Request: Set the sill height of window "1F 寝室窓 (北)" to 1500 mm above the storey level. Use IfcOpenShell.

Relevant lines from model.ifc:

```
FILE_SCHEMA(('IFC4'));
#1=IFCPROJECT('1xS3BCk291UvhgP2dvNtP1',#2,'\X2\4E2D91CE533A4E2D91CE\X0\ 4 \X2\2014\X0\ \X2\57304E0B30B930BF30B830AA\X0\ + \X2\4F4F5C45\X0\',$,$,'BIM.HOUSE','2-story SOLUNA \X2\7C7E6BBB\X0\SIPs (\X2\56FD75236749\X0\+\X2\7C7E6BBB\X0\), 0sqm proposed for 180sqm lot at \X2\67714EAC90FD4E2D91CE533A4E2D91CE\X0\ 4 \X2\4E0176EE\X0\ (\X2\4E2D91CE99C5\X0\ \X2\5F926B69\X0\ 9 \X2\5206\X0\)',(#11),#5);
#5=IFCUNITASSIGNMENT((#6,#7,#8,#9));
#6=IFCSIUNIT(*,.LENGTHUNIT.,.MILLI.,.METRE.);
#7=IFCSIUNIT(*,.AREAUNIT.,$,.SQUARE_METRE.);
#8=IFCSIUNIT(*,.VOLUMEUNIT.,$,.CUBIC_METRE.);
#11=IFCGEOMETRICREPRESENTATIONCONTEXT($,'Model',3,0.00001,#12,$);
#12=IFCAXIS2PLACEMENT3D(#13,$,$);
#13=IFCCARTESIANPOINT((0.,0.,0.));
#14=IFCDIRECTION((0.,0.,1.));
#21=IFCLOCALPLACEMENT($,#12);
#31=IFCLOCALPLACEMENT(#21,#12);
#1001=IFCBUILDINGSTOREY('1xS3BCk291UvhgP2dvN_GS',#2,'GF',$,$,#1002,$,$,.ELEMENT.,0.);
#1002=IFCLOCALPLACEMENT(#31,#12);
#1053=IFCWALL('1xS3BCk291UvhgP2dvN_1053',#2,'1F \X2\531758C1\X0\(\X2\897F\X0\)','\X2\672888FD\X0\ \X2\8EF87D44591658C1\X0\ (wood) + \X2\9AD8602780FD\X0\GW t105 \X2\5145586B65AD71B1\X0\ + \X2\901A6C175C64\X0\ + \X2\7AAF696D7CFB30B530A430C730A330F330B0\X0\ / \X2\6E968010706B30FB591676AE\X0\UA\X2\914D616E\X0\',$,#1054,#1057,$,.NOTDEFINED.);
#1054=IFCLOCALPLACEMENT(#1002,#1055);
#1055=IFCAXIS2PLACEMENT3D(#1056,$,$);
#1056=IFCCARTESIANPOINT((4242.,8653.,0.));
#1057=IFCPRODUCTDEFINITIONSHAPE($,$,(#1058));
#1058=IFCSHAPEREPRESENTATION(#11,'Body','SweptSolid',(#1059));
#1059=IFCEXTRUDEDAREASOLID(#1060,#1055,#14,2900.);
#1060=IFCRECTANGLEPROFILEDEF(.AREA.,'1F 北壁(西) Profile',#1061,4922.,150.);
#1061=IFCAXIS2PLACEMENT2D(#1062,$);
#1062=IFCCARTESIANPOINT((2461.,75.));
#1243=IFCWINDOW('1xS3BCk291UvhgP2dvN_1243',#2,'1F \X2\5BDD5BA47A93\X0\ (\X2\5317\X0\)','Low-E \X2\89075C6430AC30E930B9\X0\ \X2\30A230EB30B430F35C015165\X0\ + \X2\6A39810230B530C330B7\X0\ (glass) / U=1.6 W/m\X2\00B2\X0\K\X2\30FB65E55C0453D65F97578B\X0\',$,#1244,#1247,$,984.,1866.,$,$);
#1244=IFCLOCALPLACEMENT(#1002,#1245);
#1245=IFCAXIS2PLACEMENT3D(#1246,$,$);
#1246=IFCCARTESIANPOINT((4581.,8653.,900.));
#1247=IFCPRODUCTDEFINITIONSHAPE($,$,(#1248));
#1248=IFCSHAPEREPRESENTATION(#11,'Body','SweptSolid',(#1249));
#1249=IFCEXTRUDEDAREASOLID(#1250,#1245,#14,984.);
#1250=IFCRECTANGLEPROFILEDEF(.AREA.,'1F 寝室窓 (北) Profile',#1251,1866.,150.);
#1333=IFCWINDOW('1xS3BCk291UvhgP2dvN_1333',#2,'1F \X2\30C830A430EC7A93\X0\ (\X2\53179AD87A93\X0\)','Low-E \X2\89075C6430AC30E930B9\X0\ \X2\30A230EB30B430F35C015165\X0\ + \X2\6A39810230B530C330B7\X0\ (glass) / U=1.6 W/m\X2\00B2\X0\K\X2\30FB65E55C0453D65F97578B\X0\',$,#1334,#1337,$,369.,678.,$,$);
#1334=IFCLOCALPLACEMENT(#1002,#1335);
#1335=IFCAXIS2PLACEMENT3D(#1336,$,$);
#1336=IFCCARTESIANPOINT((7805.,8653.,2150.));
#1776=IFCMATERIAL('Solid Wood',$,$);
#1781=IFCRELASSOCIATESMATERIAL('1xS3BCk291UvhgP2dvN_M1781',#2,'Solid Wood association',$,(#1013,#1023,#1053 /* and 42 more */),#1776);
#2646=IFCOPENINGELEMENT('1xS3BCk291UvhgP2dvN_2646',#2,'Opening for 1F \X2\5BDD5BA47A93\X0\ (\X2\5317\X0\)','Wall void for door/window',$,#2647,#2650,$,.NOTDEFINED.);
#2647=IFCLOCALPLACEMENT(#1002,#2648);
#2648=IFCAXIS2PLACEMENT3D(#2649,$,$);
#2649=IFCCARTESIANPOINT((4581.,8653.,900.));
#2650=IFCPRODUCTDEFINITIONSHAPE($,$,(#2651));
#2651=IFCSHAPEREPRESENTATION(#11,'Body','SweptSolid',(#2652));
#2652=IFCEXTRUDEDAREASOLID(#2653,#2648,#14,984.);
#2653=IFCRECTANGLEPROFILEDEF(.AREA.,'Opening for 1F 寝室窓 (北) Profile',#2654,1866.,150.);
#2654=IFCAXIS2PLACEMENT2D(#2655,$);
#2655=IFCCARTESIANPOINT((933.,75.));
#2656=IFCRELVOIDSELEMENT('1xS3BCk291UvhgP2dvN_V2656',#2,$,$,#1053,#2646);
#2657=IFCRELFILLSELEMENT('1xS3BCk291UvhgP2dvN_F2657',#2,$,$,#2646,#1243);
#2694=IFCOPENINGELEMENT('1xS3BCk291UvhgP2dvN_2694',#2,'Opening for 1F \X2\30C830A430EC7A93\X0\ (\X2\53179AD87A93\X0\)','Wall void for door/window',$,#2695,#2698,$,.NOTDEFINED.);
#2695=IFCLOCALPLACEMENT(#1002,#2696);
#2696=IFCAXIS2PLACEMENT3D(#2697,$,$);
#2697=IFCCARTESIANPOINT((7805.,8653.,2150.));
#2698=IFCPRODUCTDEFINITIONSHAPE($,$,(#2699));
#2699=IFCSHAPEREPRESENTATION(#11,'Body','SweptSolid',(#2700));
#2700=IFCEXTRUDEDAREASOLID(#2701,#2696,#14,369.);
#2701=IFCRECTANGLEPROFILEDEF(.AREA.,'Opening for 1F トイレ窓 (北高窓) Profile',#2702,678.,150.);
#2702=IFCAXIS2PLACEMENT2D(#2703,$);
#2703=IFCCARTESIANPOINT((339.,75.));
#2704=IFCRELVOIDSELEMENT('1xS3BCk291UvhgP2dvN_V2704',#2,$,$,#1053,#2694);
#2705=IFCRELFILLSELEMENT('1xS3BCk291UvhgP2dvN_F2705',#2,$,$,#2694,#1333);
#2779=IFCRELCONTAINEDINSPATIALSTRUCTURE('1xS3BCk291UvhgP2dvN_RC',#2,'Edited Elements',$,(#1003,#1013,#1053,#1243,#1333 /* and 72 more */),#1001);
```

```python
import numpy as np
import ifcopenshell
import ifcopenshell.api.geometry
import ifcopenshell.geom
import ifcopenshell.util.element
import ifcopenshell.util.placement
import ifcopenshell.util.shape
import ifcopenshell.util.unit

model = ifcopenshell.open("model.ifc")
unit_scale = ifcopenshell.util.unit.calculate_unit_scale(model)

window = model.by_id(1243)
opening = window.FillsVoids[0].RelatingOpeningElement
storey = ifcopenshell.util.element.get_container(window, ifc_class="IfcBuildingStorey")
level = ifcopenshell.util.placement.get_local_placement(storey.ObjectPlacement)[2, 3]

# The opening's origin need not be at the sill, so measure its lowest point.
shape = ifcopenshell.geom.create_shape(ifcopenshell.geom.settings(), opening)
bottom = ifcopenshell.util.shape.get_shape_bottom_elevation(shape, shape.geometry) / unit_scale
dz = level + 1.5 / unit_scale - bottom

shift = np.array([0.0, 0.0, dz])
# The window is not placed relative to its opening, so move both.
for product in (opening, window):
    matrix = ifcopenshell.util.placement.get_local_placement(product.ObjectPlacement)
    matrix[:3, 3] += shift
    ifcopenshell.api.geometry.edit_object_placement(model, product=product, matrix=matrix, is_si=False)

print(f"moved by {dz * unit_scale:+.3f} m")

model.write("model_rev.ifc")
```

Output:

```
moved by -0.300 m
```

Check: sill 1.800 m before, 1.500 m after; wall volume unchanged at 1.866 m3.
